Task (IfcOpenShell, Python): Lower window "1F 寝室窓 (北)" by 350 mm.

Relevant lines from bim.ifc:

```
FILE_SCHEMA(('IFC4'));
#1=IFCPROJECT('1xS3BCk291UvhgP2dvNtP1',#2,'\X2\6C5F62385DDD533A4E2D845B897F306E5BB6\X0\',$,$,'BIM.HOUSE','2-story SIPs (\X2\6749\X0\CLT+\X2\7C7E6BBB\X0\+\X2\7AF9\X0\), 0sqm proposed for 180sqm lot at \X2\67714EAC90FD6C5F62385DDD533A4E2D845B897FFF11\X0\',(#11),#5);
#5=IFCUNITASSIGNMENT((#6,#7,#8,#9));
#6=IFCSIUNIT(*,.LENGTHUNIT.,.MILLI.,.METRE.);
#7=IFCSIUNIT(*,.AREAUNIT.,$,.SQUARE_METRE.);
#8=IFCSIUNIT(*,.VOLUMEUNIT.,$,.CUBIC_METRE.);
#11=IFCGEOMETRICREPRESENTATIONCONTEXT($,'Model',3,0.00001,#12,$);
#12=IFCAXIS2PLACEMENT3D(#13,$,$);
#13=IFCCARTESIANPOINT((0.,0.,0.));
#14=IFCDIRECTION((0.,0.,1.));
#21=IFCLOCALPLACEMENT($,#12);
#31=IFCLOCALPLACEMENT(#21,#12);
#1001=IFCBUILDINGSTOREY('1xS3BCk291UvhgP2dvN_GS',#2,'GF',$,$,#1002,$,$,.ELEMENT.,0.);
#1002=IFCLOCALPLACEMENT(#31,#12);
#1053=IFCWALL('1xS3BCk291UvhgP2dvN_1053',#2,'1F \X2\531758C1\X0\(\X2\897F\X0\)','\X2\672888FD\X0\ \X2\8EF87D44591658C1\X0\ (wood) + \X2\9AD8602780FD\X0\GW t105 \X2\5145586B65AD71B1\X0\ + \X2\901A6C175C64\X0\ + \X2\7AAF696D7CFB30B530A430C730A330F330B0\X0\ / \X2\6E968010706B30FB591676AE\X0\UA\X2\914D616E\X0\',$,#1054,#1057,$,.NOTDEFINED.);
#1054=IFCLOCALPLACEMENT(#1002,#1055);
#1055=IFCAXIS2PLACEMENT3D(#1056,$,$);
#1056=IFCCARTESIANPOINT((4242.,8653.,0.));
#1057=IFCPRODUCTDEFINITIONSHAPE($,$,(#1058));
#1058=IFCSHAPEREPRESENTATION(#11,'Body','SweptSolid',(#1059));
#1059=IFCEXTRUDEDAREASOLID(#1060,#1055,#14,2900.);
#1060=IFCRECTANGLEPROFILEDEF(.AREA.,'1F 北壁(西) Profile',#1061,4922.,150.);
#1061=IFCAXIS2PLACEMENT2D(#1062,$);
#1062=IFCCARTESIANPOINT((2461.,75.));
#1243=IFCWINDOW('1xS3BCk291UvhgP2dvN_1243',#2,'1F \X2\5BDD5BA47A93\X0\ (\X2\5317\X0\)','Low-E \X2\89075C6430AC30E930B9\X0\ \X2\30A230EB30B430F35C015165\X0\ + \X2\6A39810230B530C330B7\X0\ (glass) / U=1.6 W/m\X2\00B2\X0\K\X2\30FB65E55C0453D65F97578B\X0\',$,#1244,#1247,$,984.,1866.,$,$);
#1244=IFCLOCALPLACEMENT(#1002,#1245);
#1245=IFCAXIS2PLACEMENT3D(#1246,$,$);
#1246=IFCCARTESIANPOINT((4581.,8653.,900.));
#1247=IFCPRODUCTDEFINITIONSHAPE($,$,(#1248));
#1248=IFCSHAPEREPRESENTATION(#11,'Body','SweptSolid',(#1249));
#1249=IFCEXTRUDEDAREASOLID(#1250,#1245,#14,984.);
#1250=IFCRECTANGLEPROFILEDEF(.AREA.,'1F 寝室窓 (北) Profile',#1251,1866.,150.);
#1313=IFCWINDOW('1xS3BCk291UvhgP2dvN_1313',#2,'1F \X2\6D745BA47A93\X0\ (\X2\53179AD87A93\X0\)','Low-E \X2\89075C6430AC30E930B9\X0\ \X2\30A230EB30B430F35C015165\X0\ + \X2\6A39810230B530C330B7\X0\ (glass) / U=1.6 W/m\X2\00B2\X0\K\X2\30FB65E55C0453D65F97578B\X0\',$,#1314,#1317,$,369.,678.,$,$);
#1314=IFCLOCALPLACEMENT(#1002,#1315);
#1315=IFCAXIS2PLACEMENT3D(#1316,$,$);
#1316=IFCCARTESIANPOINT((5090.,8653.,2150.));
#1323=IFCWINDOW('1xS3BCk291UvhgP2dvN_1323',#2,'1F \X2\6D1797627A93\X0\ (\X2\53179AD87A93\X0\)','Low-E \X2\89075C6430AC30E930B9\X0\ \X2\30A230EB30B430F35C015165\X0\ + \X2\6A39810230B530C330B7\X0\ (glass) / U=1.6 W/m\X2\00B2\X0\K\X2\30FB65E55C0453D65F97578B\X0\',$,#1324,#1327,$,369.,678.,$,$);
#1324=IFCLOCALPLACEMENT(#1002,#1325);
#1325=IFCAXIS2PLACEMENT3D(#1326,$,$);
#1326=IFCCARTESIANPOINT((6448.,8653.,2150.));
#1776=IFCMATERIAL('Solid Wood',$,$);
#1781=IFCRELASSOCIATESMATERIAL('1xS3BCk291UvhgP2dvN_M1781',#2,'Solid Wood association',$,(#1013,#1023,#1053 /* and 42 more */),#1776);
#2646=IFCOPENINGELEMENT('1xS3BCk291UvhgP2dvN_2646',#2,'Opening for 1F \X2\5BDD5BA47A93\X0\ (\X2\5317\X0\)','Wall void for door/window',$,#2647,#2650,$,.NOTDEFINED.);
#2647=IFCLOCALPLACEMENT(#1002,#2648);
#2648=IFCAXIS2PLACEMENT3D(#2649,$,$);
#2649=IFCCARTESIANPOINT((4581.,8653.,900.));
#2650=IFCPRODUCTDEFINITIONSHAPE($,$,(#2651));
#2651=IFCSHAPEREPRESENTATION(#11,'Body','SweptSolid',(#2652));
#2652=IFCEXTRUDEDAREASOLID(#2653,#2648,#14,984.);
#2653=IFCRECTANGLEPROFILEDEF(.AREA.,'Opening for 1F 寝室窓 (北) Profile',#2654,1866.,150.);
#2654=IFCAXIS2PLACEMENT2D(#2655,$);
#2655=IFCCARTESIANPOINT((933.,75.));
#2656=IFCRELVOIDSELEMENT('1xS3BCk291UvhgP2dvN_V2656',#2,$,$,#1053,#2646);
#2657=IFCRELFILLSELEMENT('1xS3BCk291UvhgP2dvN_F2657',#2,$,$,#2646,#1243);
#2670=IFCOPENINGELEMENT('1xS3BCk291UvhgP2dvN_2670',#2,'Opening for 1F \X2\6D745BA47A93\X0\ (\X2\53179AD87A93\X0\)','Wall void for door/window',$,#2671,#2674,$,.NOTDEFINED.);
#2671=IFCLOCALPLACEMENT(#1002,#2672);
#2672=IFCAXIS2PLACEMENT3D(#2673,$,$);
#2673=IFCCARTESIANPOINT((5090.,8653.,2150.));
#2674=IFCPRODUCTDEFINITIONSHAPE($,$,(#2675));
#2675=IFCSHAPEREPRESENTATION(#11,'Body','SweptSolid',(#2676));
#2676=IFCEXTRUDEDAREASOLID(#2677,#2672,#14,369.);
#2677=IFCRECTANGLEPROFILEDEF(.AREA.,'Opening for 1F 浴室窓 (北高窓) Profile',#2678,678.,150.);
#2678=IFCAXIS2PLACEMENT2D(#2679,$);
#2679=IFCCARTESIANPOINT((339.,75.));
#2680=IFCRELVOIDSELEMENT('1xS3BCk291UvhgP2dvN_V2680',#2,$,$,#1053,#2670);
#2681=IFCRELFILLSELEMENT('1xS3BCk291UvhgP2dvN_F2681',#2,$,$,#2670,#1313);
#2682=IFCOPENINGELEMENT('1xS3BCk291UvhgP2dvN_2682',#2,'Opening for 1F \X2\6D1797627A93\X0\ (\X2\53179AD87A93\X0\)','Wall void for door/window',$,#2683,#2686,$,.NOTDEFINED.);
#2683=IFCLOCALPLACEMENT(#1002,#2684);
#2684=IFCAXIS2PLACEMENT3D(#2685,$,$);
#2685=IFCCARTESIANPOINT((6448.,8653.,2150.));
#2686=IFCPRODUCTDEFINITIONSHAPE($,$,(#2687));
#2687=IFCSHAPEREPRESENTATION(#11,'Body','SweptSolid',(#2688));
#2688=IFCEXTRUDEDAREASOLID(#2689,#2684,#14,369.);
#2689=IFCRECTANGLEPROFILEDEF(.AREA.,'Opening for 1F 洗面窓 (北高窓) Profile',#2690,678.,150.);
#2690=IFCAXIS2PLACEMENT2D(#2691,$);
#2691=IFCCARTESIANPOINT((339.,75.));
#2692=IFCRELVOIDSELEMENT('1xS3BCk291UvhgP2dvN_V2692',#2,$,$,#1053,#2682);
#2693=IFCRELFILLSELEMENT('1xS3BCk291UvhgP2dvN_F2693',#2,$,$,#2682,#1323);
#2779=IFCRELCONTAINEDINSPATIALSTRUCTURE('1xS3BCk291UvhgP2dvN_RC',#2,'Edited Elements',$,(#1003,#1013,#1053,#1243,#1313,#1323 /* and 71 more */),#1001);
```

```python
import numpy as np
import ifcopenshell
import ifcopenshell.api.geometry
import ifcopenshell.util.placement
import ifcopenshell.util.unit

model = ifcopenshell.open("bim.ifc")
unit_scale = ifcopenshell.util.unit.calculate_unit_scale(model)

window = model.by_guid("1xS3BCk291UvhgP2dvN_1243")
opening = window.FillsVoids[0].RelatingOpeningElement
dz = -0.35 / unit_scale

shift = np.array([0.0, 0.0, dz])
# The window is not placed relative to its opening, so move both.
for product in (opening, window):
    matrix = ifcopenshell.util.placement.get_local_placement(product.ObjectPlacement)
    matrix[:3, 3] += shift
    ifcopenshell.api.geometry.edit_object_placement(model, product=product, matrix=matrix, is_si=False)

print(f"moved by {dz * unit_scale:+.3f} m")

model.write("bim_v2.ifc")
```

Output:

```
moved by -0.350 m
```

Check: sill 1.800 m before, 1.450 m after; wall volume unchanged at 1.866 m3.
